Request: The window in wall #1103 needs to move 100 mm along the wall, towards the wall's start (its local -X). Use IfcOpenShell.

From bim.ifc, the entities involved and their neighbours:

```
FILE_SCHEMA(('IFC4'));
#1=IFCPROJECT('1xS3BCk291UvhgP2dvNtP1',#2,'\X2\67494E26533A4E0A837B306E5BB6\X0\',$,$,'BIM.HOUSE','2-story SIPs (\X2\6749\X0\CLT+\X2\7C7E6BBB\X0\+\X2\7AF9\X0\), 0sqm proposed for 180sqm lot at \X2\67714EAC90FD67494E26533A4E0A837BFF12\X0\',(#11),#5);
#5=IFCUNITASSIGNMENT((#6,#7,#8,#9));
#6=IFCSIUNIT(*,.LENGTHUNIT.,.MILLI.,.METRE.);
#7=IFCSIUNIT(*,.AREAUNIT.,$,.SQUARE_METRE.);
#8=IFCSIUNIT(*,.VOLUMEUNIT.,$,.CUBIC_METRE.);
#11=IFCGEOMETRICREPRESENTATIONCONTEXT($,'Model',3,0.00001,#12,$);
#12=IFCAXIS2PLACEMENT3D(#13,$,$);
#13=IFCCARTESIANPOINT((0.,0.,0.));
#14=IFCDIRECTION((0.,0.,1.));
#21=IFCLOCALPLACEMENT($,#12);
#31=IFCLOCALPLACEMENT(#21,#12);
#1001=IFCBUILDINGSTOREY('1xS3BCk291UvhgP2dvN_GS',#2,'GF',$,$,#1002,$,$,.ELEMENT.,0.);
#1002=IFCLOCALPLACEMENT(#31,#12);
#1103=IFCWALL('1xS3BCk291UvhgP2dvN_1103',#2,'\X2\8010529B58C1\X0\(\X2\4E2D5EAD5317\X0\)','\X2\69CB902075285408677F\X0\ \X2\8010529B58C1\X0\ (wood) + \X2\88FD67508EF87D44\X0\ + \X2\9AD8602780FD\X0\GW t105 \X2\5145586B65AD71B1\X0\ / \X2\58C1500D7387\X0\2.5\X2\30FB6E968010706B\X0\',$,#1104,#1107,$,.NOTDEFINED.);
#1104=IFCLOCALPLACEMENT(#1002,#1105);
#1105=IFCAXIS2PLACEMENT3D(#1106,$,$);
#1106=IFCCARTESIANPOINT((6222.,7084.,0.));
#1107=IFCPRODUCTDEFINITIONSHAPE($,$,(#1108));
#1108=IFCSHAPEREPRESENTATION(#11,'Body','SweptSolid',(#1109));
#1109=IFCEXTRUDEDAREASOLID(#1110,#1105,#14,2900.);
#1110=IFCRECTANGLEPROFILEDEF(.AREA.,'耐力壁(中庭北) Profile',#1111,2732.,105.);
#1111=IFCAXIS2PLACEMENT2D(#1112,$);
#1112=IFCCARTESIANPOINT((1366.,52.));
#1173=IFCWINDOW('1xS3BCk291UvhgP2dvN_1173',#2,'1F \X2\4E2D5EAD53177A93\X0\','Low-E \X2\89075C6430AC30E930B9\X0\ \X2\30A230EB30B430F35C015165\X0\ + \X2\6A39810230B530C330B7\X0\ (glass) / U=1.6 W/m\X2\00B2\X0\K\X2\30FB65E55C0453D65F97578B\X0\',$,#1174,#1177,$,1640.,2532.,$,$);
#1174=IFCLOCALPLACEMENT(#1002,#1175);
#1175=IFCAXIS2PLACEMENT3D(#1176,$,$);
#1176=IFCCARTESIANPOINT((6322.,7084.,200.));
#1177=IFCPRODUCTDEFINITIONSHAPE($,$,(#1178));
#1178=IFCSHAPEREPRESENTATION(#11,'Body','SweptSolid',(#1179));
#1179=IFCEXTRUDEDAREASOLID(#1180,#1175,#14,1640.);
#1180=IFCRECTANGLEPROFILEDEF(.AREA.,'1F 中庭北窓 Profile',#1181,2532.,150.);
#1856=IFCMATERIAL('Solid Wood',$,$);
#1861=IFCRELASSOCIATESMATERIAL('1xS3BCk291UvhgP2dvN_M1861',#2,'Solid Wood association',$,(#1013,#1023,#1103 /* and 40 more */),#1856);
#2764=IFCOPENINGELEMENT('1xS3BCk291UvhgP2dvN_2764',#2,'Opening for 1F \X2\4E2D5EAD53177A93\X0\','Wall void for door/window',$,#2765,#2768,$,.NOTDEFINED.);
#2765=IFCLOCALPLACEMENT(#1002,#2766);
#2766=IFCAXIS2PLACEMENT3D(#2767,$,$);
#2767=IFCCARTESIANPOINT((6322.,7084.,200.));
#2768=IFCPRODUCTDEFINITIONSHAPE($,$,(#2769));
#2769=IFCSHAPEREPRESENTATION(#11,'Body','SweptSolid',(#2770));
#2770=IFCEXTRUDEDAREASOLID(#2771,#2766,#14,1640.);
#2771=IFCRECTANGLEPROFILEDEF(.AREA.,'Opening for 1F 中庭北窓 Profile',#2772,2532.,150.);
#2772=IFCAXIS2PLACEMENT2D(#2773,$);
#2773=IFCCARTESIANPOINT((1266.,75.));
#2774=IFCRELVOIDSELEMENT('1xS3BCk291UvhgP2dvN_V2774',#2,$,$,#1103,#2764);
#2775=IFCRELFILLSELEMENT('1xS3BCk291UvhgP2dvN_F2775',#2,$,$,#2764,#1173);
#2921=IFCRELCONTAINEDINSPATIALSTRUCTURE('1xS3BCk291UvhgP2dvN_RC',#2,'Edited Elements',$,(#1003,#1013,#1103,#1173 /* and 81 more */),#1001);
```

```python
import ifcopenshell
import ifcopenshell.api.geometry
import ifcopenshell.util.placement

model = ifcopenshell.open("bim.ifc")

window = model.by_guid("1xS3BCk291UvhgP2dvN_1173")
opening = window.FillsVoids[0].RelatingOpeningElement
wall = opening.VoidsElements[0].RelatingBuildingElement

wall_matrix = ifcopenshell.util.placement.get_local_placement(wall.ObjectPlacement)
shift = wall_matrix[:3, 0] * -100.0
before = ifcopenshell.util.placement.get_local_placement(window.ObjectPlacement)[:3, 3].copy()

# The window is not placed relative to its opening, so move both.
for product in (opening, window):
    matrix = ifcopenshell.util.placement.get_local_placement(product.ObjectPlacement)
    matrix[:3, 3] += shift
    ifcopenshell.api.geometry.edit_object_placement(model, product=product, matrix=matrix, is_si=False)

after = ifcopenshell.util.placement.get_local_placement(window.ObjectPlacement)[:3, 3]
print("window moved by", (after - before).round(3) + 0.0)

model.write("bim_v2.ifc")
```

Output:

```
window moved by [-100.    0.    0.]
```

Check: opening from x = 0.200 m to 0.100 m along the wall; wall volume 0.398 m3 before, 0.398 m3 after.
